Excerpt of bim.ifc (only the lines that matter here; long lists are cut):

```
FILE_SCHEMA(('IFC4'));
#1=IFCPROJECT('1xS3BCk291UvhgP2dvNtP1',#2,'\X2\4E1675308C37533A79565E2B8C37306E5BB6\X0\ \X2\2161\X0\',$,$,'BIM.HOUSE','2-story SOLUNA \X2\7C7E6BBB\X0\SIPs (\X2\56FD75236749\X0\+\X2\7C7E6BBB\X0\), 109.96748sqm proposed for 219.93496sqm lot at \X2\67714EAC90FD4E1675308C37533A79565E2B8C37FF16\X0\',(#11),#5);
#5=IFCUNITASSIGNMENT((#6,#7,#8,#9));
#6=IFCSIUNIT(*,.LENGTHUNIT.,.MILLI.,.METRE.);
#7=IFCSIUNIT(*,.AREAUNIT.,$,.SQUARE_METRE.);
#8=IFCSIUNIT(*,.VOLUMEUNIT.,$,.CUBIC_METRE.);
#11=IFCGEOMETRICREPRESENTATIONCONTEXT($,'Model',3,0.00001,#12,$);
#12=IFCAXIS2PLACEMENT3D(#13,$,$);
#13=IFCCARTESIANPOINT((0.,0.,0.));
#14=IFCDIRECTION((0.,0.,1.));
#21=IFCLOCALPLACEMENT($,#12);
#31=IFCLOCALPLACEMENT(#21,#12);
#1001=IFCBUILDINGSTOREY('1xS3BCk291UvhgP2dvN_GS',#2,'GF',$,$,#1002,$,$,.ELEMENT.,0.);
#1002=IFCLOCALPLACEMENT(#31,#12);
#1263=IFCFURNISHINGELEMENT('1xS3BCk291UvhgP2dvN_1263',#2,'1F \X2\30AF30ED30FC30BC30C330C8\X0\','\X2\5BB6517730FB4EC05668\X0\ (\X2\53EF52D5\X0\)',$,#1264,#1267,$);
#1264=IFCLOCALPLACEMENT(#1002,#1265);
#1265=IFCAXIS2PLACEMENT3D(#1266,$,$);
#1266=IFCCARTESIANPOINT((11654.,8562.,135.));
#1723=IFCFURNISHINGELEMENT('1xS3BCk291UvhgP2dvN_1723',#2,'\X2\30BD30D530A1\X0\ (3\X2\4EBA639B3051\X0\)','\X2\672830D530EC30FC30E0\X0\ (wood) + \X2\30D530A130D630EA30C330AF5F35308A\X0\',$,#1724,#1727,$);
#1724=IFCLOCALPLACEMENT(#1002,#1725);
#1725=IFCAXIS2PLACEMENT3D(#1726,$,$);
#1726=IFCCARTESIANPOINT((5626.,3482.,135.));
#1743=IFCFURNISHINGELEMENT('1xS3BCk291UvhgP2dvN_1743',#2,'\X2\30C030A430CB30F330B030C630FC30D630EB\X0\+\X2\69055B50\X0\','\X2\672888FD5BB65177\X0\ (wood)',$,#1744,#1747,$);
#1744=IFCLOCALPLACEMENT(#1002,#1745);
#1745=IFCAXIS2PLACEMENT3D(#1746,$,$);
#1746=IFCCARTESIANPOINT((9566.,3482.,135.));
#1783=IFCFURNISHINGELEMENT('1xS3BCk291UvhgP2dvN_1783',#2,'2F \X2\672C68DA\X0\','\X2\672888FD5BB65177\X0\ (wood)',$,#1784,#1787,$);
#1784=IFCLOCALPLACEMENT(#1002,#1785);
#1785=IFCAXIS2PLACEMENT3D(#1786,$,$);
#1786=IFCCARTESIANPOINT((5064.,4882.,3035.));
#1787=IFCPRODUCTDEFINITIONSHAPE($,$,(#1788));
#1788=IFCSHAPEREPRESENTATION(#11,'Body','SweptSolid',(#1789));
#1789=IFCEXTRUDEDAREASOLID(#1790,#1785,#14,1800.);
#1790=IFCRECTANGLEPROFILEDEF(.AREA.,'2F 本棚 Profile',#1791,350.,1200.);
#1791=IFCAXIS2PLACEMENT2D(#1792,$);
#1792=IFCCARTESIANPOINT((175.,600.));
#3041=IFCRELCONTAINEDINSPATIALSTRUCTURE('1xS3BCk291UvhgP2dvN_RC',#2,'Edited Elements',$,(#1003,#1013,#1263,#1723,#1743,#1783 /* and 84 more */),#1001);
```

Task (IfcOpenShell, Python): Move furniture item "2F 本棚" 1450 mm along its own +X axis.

```python
import ifcopenshell
import ifcopenshell.api.geometry
import ifcopenshell.util.placement

model = ifcopenshell.open("bim.ifc")

item = model.by_id(1783)
matrix = ifcopenshell.util.placement.get_local_placement(item.ObjectPlacement)
matrix[:3, 3] += matrix[:3, 0] * 1450.0
ifcopenshell.api.geometry.edit_object_placement(model, product=item, matrix=matrix, is_si=False)

print(ifcopenshell.util.placement.get_local_placement(item.ObjectPlacement).round(3) + 0.0)

model.write("bim_updated.ifc")
```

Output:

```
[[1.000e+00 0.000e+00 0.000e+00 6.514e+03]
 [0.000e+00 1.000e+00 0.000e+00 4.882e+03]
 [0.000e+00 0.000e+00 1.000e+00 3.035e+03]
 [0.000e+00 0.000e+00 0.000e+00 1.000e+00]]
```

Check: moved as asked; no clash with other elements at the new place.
